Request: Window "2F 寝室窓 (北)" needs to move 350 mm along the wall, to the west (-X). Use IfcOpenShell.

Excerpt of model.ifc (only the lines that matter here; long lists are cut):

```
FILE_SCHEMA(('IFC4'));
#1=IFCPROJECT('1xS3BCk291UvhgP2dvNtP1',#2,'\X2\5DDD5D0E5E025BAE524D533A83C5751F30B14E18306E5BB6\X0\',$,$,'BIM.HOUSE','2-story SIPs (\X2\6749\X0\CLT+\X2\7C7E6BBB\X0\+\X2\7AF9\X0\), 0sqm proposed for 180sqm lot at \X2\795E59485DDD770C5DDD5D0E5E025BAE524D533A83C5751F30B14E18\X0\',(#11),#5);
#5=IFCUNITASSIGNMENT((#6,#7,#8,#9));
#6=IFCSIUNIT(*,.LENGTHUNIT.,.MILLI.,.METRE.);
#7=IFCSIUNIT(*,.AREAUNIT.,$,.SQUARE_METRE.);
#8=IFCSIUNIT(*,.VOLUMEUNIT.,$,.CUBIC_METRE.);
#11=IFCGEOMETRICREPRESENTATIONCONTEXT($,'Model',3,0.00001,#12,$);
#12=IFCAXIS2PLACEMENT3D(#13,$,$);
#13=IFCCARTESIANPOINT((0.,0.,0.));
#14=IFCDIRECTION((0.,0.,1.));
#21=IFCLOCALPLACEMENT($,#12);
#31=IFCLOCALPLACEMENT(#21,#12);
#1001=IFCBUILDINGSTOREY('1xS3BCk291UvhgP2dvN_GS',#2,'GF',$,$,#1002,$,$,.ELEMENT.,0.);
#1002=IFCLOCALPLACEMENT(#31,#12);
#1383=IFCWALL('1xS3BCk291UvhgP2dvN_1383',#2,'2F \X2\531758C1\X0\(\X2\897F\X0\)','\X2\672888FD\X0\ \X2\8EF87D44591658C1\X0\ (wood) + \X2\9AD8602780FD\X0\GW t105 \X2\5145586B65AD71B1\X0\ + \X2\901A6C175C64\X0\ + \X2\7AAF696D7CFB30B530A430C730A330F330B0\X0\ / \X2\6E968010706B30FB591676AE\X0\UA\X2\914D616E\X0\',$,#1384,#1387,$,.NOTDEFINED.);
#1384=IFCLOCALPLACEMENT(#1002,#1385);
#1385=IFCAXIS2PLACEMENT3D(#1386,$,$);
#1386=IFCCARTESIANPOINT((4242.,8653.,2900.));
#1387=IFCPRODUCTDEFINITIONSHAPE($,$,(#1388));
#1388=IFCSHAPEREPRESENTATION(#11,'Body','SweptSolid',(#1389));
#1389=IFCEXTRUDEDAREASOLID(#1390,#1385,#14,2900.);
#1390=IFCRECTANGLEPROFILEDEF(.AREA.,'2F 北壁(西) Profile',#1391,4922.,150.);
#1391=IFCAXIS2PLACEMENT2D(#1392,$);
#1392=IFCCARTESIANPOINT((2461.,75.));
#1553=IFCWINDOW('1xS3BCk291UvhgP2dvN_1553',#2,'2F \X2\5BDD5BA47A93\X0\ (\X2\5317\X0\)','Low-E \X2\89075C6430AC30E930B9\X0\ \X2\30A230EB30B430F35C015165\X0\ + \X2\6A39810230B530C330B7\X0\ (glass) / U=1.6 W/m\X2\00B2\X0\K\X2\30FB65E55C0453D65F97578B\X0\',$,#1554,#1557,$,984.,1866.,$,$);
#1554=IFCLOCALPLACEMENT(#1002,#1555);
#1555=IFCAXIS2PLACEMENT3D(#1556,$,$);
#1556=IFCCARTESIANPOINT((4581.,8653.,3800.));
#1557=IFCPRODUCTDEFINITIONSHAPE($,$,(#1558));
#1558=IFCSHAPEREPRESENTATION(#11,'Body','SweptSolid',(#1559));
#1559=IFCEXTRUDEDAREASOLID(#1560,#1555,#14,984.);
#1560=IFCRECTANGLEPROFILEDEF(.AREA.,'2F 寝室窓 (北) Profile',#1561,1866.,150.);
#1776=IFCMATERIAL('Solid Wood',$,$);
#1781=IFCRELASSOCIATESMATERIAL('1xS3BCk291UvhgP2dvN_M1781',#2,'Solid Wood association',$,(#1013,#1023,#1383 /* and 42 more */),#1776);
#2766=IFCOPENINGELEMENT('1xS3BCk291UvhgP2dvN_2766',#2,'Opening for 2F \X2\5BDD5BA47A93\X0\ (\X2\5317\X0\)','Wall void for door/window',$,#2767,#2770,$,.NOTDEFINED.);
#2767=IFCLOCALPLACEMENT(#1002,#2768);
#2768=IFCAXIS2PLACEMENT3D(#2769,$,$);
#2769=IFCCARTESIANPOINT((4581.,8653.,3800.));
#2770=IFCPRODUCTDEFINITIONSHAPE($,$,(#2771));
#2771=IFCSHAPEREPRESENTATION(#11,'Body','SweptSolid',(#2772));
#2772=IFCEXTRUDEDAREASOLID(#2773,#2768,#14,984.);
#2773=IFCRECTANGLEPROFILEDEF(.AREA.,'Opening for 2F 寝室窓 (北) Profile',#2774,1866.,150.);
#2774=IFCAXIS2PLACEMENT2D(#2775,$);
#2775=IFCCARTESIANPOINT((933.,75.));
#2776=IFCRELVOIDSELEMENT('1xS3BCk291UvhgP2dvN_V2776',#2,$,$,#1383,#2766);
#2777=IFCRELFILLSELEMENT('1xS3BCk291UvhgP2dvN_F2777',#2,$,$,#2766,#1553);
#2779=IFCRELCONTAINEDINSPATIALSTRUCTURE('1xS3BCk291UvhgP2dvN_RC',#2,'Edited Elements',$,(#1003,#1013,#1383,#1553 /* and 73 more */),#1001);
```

```python
import ifcopenshell
import ifcopenshell.api.geometry
import ifcopenshell.util.placement

model = ifcopenshell.open("model.ifc")

window = model.by_guid("1xS3BCk291UvhgP2dvN_1553")
opening = window.FillsVoids[0].RelatingOpeningElement
wall = opening.VoidsElements[0].RelatingBuildingElement

wall_matrix = ifcopenshell.util.placement.get_local_placement(wall.ObjectPlacement)
shift = wall_matrix[:3, 0] * -350.0
before = ifcopenshell.util.placement.get_local_placement(window.ObjectPlacement)[:3, 3].copy()

# The window is not placed relative to its opening, so move both.
for product in (opening, window):
    matrix = ifcopenshell.util.placement.get_local_placement(product.ObjectPlacement)
    matrix[:3, 3] += shift
    ifcopenshell.api.geometry.edit_object_placement(model, product=product, matrix=matrix, is_si=False)

after = ifcopenshell.util.placement.get_local_placement(window.ObjectPlacement)[:3, 3]
print("window moved by", (after - before).round(3) + 0.0)

model.write("model_edited.ifc")
```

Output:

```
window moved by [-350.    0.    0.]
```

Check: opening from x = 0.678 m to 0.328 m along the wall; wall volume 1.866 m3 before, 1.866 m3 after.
